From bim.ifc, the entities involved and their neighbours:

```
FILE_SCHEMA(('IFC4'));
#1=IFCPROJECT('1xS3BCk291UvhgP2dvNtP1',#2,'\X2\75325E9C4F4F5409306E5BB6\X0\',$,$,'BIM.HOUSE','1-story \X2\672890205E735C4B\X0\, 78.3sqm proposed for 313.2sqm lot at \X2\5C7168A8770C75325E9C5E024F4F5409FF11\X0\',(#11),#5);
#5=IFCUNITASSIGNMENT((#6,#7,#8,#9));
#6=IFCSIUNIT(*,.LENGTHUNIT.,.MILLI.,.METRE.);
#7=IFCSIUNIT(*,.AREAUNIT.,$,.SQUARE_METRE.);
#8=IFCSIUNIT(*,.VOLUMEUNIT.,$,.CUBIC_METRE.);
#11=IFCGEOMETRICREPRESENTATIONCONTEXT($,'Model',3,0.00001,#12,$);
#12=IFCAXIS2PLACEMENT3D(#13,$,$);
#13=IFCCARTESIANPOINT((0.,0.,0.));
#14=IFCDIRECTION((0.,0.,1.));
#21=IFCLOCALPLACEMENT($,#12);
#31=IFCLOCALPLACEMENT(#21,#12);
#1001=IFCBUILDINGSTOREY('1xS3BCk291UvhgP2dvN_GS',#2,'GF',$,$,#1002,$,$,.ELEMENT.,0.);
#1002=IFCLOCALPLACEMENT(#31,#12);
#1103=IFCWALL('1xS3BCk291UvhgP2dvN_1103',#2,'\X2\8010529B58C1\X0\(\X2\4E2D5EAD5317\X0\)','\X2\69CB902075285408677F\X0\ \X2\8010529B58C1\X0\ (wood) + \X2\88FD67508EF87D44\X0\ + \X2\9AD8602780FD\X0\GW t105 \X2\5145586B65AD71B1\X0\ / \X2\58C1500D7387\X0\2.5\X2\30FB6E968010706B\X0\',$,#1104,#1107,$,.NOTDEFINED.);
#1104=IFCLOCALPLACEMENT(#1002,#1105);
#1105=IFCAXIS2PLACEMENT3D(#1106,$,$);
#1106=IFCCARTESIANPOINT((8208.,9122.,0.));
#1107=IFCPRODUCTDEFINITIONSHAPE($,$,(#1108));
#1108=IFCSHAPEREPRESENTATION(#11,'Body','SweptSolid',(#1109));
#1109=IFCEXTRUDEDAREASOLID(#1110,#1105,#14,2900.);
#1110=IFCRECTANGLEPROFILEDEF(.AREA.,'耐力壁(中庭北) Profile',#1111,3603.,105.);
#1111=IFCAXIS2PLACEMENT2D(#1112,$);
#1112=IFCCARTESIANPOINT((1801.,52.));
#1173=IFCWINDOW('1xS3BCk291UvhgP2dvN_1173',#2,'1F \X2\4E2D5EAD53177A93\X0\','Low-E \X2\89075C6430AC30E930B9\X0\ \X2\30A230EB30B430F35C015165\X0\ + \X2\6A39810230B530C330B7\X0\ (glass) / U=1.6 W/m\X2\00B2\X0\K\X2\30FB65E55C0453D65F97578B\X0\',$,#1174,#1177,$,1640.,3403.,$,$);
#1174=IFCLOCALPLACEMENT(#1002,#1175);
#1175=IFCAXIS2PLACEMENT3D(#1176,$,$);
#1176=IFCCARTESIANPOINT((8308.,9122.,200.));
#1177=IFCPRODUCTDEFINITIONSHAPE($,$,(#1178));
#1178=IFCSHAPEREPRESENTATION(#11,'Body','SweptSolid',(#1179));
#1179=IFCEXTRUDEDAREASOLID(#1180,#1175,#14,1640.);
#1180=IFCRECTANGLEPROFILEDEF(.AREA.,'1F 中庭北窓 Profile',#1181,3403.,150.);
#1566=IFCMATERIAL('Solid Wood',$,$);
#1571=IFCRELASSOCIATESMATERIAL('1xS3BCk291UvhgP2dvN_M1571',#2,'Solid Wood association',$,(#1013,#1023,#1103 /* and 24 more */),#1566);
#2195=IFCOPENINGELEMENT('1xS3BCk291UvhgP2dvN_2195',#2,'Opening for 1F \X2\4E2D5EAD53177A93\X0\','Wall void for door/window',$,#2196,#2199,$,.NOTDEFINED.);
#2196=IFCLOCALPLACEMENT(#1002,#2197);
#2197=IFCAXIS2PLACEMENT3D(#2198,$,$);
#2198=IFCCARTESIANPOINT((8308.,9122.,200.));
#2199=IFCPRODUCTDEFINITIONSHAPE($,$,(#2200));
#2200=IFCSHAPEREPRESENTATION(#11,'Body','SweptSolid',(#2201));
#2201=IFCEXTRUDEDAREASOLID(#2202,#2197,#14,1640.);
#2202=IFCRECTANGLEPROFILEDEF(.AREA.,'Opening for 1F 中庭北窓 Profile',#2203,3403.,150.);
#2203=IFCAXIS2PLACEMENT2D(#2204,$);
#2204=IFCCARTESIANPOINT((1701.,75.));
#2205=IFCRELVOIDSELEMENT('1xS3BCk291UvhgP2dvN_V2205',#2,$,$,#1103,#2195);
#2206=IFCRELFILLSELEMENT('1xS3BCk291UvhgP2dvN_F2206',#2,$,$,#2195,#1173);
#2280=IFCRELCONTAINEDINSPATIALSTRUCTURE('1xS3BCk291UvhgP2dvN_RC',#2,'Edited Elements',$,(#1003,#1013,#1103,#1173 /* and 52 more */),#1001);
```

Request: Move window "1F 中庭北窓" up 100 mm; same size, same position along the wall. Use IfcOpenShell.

```python
import numpy as np
import ifcopenshell
import ifcopenshell.api.geometry
import ifcopenshell.util.placement
import ifcopenshell.util.unit

model = ifcopenshell.open("bim.ifc")
unit_scale = ifcopenshell.util.unit.calculate_unit_scale(model)

window = model.by_guid("1xS3BCk291UvhgP2dvN_1173")
opening = window.FillsVoids[0].RelatingOpeningElement
dz = 0.1 / unit_scale

shift = np.array([0.0, 0.0, dz])
# The window is not placed relative to its opening, so move both.
for product in (opening, window):
    matrix = ifcopenshell.util.placement.get_local_placement(product.ObjectPlacement)
    matrix[:3, 3] += shift
    ifcopenshell.api.geometry.edit_object_placement(model, product=product, matrix=matrix, is_si=False)

print(f"moved by {dz * unit_scale:+.3f} m")

model.write("bim_edited.ifc")
```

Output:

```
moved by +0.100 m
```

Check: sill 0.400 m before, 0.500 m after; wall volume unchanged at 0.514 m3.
